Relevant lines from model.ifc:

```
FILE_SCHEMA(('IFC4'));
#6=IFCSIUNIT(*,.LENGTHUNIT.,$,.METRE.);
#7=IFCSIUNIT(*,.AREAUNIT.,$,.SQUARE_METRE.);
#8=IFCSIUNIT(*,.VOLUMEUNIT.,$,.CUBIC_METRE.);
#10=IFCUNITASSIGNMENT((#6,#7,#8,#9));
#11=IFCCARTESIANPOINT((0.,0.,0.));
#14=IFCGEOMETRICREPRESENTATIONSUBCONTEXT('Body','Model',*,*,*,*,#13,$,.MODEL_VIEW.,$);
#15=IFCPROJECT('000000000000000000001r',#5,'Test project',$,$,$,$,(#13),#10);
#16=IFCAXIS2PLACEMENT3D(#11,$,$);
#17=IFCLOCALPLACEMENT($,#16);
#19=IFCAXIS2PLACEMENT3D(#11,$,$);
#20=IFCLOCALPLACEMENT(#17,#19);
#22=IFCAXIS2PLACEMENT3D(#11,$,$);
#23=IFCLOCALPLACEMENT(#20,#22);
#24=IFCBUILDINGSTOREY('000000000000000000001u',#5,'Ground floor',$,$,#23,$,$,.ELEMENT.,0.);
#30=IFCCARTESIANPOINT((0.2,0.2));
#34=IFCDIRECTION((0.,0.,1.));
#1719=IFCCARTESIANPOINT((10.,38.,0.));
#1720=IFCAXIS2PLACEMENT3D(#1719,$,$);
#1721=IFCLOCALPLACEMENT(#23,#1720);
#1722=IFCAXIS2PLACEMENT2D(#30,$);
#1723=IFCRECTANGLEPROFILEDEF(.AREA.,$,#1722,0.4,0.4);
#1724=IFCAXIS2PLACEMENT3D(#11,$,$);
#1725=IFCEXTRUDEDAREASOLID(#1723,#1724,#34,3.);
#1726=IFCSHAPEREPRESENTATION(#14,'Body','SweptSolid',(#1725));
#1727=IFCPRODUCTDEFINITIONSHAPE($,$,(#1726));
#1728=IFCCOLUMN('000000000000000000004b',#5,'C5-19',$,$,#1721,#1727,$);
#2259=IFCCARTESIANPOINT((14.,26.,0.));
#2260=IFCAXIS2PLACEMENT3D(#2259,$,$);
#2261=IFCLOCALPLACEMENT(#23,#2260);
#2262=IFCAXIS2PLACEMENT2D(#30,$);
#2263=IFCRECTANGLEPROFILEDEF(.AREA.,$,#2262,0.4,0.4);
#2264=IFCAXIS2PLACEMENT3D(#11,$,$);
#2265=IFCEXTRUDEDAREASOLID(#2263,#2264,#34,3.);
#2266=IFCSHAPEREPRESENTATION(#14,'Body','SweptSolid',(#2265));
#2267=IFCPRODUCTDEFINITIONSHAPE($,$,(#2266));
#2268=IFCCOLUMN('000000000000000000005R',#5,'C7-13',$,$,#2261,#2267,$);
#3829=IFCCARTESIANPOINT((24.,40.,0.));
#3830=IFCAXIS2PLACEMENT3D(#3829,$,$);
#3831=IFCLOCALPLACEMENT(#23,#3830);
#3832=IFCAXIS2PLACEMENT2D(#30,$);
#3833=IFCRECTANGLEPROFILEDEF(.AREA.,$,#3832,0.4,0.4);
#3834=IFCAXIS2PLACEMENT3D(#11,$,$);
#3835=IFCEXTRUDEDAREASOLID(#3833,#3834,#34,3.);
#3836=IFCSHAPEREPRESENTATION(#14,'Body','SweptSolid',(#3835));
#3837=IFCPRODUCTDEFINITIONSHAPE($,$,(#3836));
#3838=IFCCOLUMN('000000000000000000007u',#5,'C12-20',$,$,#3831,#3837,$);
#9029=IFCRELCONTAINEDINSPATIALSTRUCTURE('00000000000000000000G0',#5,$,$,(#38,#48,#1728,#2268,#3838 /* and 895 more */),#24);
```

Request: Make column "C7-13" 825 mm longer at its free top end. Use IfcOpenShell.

```python
import ifcopenshell
import ifcopenshell.util.representation

model = ifcopenshell.open("model.ifc")

member = model.by_guid("000000000000000000005R")
change = 0.825

# The extrusion runs towards the end named, so only its depth changes.
body = ifcopenshell.util.representation.get_representation(member, "Model", "Body")
solid = body.Items[0]
old_length = solid.Depth
solid.Depth += change

print(f"length {old_length:g} -> {solid.Depth:g}")

model.write("model_v2.ifc")
```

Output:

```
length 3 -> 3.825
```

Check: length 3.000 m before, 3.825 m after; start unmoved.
